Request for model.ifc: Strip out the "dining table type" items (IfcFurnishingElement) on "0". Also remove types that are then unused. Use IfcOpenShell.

First a look at what the model holds.

```python
import ifcopenshell
import ifcopenshell.util.element

model = ifcopenshell.open("model.ifc")
print(model.schema)
storey = next(s for s in model.by_type("IfcBuildingStorey") if s.Name == "0")
furniture = [e for e in ifcopenshell.util.element.get_decomposition(storey) if e.is_a("IfcFurnishingElement")]
seen = {}
for e in furniture:
    element_type = ifcopenshell.util.element.get_type(e)
    name = element_type.Name if element_type not in (None, e) else None
    seen[name] = seen.get(name, 0) + 1
for name, count in sorted(seen.items(), key=str):
    print(count, "x", name)
```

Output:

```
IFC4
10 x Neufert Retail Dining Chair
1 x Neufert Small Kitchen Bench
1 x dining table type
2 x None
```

```python
import ifcopenshell
import ifcopenshell.api.root
import ifcopenshell.util.element

model = ifcopenshell.open("model.ifc")

storey = next(s for s in model.by_type("IfcBuildingStorey") if s.Name == "0")
furniture = [e for e in ifcopenshell.util.element.get_decomposition(storey) if e.is_a("IfcFurnishingElement")]
targets = [e for e in furniture if (t := ifcopenshell.util.element.get_type(e)) not in (None, e) and t.Name == "dining table type"]
types = {ifcopenshell.util.element.get_type(e) for e in targets} - {None, *targets}

for e in targets:
    ifcopenshell.api.root.remove_product(model, product=e)
print(len(targets), "removed")

unused = [t for t in types if not ifcopenshell.util.element.get_types(t)]
for t in unused:
    ifcopenshell.api.root.remove_product(model, product=t)
print(len(unused), "unused types removed")

model.write("model_updated.ifc")
```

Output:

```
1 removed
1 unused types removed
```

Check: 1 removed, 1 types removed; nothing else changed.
